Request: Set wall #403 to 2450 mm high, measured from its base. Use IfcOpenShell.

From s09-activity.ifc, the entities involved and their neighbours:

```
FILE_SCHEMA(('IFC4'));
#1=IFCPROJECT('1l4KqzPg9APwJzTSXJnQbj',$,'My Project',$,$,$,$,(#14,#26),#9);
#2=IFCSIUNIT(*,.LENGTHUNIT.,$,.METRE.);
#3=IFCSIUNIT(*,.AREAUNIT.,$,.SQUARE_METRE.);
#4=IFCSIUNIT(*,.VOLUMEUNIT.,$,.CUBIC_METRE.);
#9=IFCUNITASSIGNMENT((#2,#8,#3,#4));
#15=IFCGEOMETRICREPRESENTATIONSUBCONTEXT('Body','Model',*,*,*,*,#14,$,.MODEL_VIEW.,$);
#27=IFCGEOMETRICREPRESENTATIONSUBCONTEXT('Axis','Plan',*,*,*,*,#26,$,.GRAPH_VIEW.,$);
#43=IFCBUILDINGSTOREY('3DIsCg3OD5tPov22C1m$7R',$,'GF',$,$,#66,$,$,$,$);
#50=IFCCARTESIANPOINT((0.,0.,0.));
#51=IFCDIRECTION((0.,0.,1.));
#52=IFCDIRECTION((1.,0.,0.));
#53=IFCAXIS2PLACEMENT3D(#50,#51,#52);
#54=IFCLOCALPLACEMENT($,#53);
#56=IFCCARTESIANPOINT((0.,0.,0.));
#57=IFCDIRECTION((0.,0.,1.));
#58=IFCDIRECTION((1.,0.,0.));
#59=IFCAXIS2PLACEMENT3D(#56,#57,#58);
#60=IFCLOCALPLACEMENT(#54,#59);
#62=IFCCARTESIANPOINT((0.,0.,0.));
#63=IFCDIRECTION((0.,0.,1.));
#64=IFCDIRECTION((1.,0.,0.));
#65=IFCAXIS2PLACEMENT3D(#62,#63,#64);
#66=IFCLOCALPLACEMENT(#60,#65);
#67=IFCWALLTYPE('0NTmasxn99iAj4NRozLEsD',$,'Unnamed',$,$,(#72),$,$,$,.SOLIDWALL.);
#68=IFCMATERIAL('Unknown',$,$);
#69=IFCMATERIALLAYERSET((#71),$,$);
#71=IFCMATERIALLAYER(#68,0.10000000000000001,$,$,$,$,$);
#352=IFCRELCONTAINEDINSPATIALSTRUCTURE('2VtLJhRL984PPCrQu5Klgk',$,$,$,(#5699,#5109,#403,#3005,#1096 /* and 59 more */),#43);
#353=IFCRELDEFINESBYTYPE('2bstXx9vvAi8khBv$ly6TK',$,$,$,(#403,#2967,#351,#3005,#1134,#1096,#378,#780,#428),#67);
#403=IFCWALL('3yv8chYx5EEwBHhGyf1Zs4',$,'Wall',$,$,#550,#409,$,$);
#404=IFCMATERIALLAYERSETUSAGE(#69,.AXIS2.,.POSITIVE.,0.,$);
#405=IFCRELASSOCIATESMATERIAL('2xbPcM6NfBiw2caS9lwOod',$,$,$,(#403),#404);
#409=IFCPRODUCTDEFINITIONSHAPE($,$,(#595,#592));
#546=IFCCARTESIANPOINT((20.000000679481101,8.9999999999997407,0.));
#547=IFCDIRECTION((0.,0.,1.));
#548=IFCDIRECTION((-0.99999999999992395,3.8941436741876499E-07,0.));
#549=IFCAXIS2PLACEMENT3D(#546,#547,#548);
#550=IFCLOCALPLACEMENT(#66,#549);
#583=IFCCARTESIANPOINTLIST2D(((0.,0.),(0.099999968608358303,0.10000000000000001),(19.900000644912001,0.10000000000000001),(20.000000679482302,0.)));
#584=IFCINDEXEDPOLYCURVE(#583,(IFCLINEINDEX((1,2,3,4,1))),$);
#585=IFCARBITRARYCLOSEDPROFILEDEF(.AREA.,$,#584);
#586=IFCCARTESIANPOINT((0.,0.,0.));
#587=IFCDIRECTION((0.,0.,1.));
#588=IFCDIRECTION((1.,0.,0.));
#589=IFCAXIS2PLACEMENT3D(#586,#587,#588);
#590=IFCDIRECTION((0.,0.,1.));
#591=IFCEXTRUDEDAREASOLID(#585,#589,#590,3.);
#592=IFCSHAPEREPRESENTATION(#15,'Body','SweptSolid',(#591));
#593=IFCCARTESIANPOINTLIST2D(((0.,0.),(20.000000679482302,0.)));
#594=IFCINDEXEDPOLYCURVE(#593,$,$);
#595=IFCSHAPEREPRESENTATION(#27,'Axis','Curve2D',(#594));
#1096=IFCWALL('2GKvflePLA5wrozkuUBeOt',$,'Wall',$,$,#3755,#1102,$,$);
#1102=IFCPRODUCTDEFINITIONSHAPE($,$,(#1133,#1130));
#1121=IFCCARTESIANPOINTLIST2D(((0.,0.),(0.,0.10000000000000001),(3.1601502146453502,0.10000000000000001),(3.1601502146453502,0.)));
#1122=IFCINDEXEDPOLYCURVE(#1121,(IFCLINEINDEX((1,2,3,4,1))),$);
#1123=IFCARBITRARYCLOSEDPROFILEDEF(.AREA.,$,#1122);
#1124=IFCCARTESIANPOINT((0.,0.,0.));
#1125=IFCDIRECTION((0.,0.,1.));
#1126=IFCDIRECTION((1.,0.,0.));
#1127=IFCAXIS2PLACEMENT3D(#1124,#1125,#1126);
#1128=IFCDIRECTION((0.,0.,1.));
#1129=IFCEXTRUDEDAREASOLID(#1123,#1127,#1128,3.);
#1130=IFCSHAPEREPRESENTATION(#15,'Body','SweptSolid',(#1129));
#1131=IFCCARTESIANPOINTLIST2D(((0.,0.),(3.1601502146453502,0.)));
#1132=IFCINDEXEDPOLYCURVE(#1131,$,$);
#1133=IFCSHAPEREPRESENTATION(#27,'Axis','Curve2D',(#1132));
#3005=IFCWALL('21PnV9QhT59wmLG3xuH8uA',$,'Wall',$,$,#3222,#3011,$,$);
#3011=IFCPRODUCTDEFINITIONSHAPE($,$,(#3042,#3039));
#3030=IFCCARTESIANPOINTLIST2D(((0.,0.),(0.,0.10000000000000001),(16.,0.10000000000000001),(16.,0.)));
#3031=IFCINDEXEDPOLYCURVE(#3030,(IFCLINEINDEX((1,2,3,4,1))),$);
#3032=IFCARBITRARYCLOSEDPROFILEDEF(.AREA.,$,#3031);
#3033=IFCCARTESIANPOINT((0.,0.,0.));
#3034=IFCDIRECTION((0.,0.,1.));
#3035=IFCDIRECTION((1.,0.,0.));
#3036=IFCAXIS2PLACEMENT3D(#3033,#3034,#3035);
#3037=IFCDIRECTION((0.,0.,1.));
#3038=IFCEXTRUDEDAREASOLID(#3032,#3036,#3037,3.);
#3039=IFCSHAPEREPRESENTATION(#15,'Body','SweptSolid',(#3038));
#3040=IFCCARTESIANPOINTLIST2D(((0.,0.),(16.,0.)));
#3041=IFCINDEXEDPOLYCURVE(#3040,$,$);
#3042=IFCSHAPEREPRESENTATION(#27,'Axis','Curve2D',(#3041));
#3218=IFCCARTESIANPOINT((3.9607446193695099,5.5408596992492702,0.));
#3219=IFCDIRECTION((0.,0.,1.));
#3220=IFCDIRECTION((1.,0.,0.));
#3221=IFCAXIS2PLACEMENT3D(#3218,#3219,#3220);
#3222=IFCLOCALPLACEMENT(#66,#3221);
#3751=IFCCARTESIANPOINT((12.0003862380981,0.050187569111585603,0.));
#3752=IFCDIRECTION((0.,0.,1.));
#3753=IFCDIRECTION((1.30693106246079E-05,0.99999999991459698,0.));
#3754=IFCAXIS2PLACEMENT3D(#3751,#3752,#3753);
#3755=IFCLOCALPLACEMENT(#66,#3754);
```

```python
import ifcopenshell
import ifcopenshell.geom
import ifcopenshell.util.representation
import ifcopenshell.util.shape
import ifcopenshell.util.unit

model = ifcopenshell.open("s09-activity.ifc")
unit_scale = ifcopenshell.util.unit.calculate_unit_scale(model)
settings = ifcopenshell.geom.settings()


def volume(element):
    """Net volume in cubic metres, openings subtracted."""
    shape = ifcopenshell.geom.create_shape(settings, element)
    return ifcopenshell.util.shape.get_volume(shape.geometry)


wall = model.by_guid("3yv8chYx5EEwBHhGyf1Zs4")
before = volume(wall)

body = ifcopenshell.util.representation.get_representation(wall, "Model", "Body")
solid = body.Items[0]
old_height = solid.Depth
solid.Depth = 2.45 / unit_scale
after = volume(wall)

print(f"height {old_height:g} -> {solid.Depth:g}, volume {before:.3f} -> {after:.3f} m3")

model.write("s09-activity_rev.ifc")
```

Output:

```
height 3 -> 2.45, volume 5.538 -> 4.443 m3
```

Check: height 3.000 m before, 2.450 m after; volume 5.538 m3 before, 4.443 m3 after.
